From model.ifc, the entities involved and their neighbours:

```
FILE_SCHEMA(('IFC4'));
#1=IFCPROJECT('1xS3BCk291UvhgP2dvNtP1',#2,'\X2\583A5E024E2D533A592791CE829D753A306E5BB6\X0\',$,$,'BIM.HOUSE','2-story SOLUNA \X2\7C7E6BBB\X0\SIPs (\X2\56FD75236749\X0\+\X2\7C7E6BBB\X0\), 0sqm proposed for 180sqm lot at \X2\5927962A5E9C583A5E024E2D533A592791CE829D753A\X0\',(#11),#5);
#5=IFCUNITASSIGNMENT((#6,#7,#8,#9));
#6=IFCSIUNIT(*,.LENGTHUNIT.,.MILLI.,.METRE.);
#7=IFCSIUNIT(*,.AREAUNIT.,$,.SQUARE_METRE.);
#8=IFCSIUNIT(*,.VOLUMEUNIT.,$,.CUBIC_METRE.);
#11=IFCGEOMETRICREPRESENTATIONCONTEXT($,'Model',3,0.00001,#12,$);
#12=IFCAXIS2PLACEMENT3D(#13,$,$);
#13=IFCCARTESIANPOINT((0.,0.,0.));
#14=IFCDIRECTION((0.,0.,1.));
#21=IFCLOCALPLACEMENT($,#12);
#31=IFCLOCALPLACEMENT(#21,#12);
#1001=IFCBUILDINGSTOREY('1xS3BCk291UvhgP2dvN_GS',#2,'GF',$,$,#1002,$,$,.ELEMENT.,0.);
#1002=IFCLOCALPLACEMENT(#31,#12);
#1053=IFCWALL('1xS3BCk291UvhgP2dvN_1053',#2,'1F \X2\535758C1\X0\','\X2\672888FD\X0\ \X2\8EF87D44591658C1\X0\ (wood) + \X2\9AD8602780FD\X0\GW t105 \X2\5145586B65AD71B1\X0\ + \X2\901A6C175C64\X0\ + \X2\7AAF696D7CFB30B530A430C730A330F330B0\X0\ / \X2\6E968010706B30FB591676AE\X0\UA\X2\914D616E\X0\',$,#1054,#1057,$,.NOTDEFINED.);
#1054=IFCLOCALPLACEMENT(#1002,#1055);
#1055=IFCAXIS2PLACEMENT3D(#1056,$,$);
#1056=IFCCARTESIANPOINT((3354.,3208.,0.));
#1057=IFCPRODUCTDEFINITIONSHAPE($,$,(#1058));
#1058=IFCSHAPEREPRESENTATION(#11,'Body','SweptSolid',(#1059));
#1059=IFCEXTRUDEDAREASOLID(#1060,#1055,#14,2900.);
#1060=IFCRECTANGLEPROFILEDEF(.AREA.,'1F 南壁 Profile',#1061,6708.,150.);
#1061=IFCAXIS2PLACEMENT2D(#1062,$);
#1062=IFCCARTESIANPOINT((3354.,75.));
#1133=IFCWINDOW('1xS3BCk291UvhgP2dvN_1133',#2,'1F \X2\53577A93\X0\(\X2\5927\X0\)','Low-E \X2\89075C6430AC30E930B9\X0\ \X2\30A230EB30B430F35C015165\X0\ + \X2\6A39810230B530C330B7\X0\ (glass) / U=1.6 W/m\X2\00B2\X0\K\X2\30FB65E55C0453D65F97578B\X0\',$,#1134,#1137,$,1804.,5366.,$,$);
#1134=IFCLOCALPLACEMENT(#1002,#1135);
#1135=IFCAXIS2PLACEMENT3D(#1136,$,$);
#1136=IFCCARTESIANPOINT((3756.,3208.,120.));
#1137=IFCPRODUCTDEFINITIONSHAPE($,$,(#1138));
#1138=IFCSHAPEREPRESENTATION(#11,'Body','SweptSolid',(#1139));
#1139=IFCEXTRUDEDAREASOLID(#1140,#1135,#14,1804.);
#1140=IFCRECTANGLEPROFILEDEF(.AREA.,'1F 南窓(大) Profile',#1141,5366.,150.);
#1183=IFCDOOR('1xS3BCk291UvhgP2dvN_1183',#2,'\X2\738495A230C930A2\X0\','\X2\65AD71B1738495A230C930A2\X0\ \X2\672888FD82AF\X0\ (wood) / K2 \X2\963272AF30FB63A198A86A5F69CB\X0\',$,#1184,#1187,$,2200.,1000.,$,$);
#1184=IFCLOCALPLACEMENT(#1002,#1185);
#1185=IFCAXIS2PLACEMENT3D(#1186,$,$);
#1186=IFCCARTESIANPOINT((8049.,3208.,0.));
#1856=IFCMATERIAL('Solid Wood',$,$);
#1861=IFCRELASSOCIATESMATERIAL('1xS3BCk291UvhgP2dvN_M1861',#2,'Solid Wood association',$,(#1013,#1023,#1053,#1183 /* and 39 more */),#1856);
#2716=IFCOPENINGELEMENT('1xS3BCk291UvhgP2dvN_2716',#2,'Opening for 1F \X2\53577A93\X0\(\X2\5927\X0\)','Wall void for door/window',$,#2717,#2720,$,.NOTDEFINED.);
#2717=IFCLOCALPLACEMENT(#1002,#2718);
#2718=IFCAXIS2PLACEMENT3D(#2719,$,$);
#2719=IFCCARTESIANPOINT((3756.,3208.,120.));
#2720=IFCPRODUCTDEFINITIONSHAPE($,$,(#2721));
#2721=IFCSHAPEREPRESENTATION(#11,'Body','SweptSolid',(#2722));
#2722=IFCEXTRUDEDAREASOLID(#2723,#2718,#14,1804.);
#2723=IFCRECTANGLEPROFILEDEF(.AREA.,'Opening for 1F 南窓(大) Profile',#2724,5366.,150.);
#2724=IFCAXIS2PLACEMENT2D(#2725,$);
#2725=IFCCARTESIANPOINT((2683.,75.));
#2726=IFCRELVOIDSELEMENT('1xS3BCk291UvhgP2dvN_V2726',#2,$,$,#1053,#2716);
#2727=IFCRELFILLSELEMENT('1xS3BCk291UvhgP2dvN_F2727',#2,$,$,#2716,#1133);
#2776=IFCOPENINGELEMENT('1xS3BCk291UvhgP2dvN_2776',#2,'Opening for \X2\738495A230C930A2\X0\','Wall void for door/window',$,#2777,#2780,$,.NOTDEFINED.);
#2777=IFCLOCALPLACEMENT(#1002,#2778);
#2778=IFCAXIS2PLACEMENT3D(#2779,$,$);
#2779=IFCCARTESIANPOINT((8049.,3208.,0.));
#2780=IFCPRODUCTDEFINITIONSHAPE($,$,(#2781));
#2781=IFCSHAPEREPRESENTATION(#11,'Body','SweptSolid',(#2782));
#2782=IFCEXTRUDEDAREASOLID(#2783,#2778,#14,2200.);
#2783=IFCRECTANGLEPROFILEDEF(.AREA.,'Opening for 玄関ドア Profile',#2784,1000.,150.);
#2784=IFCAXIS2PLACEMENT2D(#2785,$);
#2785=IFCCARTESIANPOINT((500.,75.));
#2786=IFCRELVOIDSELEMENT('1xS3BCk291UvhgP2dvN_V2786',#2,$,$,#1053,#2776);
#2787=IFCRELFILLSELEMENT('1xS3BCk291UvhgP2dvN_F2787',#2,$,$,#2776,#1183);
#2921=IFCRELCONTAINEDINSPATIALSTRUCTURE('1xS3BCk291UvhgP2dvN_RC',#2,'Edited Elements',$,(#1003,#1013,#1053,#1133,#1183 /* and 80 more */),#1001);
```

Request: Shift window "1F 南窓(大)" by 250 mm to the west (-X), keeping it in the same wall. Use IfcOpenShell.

```python
import ifcopenshell
import ifcopenshell.api.geometry
import ifcopenshell.util.placement
import ifcopenshell.util.unit

model = ifcopenshell.open("model.ifc")
unit_scale = ifcopenshell.util.unit.calculate_unit_scale(model)

window = model.by_guid("1xS3BCk291UvhgP2dvN_1133")
opening = window.FillsVoids[0].RelatingOpeningElement
wall = opening.VoidsElements[0].RelatingBuildingElement

wall_matrix = ifcopenshell.util.placement.get_local_placement(wall.ObjectPlacement)
shift = wall_matrix[:3, 0] * -0.25 / unit_scale
before = ifcopenshell.util.placement.get_local_placement(window.ObjectPlacement)[:3, 3].copy()

# The window is not placed relative to its opening, so move both.
for product in (opening, window):
    matrix = ifcopenshell.util.placement.get_local_placement(product.ObjectPlacement)
    matrix[:3, 3] += shift
    ifcopenshell.api.geometry.edit_object_placement(model, product=product, matrix=matrix, is_si=False)

after = ifcopenshell.util.placement.get_local_placement(window.ObjectPlacement)[:3, 3]
print("window moved by", (after - before).round(3) + 0.0)

model.write("model_updated.ifc")
```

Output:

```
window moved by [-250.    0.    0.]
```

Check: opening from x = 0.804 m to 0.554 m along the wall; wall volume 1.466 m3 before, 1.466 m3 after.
